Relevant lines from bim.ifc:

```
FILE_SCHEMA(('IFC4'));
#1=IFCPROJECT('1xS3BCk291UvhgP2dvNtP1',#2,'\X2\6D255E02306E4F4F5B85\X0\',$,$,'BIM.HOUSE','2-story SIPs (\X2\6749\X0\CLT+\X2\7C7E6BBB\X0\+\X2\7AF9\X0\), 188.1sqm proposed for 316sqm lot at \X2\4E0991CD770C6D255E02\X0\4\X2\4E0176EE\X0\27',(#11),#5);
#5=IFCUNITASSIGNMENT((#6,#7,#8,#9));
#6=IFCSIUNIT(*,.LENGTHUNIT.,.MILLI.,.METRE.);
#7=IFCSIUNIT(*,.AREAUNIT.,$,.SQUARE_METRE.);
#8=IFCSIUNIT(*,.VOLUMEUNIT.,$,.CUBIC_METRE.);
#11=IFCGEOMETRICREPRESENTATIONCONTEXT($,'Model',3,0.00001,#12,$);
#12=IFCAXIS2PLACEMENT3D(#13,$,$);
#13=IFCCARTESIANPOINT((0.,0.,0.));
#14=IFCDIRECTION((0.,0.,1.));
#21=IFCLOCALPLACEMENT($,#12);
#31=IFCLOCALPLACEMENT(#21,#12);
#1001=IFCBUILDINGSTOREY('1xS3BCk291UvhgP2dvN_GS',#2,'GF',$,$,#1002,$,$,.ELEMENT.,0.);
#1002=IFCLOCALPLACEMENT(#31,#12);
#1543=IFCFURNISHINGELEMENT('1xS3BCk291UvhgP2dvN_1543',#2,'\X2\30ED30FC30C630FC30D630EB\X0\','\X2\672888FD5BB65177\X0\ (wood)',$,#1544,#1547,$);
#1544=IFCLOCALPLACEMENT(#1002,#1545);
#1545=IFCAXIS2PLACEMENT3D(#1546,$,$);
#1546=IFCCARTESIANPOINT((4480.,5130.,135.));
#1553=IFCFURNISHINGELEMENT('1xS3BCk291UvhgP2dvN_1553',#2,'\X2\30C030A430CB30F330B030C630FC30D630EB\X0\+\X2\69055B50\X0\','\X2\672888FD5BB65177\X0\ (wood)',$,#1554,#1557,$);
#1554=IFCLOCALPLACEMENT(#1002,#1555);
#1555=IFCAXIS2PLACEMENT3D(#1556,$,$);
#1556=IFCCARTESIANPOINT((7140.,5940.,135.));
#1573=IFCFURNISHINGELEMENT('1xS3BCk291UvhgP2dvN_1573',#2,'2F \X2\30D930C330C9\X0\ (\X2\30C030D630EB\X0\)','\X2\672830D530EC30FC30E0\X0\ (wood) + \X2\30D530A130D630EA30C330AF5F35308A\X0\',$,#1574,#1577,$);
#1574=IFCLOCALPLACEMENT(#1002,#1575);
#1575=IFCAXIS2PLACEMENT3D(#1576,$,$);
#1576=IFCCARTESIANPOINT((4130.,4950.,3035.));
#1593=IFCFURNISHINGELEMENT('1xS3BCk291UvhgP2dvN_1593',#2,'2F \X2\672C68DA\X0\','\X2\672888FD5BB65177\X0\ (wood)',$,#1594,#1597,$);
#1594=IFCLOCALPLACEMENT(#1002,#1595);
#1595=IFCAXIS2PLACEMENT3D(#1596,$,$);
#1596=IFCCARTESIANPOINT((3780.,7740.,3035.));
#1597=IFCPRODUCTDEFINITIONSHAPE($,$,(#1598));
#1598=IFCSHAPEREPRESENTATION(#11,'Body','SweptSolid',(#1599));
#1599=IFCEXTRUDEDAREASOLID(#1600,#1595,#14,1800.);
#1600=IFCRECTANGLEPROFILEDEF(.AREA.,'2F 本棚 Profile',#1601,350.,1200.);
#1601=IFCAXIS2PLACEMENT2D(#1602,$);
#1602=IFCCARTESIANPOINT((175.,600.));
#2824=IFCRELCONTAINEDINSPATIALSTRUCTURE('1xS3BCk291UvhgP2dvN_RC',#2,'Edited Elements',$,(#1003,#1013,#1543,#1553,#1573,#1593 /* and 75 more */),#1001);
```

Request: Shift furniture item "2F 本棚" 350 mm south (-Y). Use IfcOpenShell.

```python
import ifcopenshell
import ifcopenshell.api.geometry
import ifcopenshell.util.placement

model = ifcopenshell.open("bim.ifc")

item = model.by_id(1593)
matrix = ifcopenshell.util.placement.get_local_placement(item.ObjectPlacement)
matrix[1, 3] -= 350.0
ifcopenshell.api.geometry.edit_object_placement(model, product=item, matrix=matrix, is_si=False)

print(ifcopenshell.util.placement.get_local_placement(item.ObjectPlacement).round(3) + 0.0)

model.write("bim_rev.ifc")
```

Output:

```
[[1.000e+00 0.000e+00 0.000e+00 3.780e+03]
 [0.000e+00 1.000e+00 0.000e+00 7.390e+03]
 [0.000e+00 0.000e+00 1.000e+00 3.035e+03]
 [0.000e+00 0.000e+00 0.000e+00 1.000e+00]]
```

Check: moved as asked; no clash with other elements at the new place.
